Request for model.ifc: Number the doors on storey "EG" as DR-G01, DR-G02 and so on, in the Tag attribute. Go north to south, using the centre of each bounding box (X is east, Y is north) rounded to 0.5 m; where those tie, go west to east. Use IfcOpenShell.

First a look at what the model holds.

```python
import ifcopenshell
import ifcopenshell.util.element
import ifcopenshell.util.placement

model = ifcopenshell.open("model.ifc")
print(model.schema)
storey = next(s for s in model.by_type("IfcBuildingStorey") if s.Name == "EG")
doors = [e for e in ifcopenshell.util.element.get_decomposition(storey) if e.is_a("IfcDoor")]
for e in sorted(doors, key=lambda e: e.id()):
    origin = ifcopenshell.util.placement.get_local_placement(e.ObjectPlacement)[:3, 3]
    print(e.id(), e.Tag, e.Name, origin.round(2) + 0.0, sep=" | ")
```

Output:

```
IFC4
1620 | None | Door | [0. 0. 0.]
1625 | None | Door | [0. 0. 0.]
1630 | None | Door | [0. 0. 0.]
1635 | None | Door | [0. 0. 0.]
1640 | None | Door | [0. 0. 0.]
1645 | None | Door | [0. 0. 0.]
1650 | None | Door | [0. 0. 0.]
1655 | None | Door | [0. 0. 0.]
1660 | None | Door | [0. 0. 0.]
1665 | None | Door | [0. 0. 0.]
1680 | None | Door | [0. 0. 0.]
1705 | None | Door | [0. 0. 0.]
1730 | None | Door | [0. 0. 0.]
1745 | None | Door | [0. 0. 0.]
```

```python
import ifcopenshell
import ifcopenshell.geom
import ifcopenshell.util.element
import ifcopenshell.util.shape

model = ifcopenshell.open("model.ifc")
settings = ifcopenshell.geom.settings()
settings.set("use-world-coords", True)


def centre(element):
    shape = ifcopenshell.geom.create_shape(settings, element)
    return ifcopenshell.util.shape.get_bbox_centroid(shape.geometry)


storey = next(s for s in model.by_type("IfcBuildingStorey") if s.Name == "EG")
doors = [e for e in ifcopenshell.util.element.get_decomposition(storey) if e.is_a("IfcDoor")]

# Insertion points can sit at a corner or the storey origin, so sort by the geometry (in metres).
centres = {e: centre(e) for e in doors}
doors.sort(key=lambda e: (-round(centres[e][1] / 0.5), centres[e][0]))

for i, e in enumerate(doors, start=1):
    number = f"DR-G{i:02d}"
    e.Tag = number
    print(e.id(), number)

model.write("model_v2.ifc")
```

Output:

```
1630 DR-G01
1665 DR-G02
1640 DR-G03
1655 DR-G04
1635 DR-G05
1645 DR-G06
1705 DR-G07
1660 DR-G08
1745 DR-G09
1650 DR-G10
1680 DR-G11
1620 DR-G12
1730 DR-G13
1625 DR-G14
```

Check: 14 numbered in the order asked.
